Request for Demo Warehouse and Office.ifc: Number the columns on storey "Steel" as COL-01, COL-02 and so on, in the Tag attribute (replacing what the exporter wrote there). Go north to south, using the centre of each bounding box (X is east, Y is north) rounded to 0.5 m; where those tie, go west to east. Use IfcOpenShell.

First a look at what the model holds.

```python
import ifcopenshell
import ifcopenshell.util.element
import ifcopenshell.util.placement

model = ifcopenshell.open("Demo Warehouse and Office.ifc")
print(model.schema)
storey = next(s for s in model.by_type("IfcBuildingStorey") if s.Name == "Steel")
columns = [e for e in ifcopenshell.util.element.get_decomposition(storey) if e.is_a("IfcColumn")]
for e in sorted(columns, key=lambda e: e.id()):
    origin = ifcopenshell.util.placement.get_local_placement(e.ObjectPlacement)[:3, 3]
    print(e.id(), e.Tag, e.Name, origin.round(2) + 0.0, sep=" | ")
```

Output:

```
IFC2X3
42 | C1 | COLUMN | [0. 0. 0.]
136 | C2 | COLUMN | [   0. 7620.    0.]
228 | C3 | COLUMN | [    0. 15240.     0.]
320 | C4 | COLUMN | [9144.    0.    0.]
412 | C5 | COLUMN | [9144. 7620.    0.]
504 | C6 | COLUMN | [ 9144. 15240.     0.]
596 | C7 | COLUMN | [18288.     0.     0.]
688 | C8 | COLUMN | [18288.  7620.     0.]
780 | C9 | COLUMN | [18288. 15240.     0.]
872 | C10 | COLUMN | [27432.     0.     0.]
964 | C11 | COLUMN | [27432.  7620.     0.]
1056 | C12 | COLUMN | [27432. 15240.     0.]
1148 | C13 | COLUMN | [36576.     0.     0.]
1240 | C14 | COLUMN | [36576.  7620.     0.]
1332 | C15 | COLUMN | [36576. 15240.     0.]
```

```python
import ifcopenshell
import ifcopenshell.geom
import ifcopenshell.util.element
import ifcopenshell.util.shape

model = ifcopenshell.open("Demo Warehouse and Office.ifc")
settings = ifcopenshell.geom.settings()
settings.set("use-world-coords", True)


def centre(element):
    shape = ifcopenshell.geom.create_shape(settings, element)
    return ifcopenshell.util.shape.get_bbox_centroid(shape.geometry)


storey = next(s for s in model.by_type("IfcBuildingStorey") if s.Name == "Steel")
columns = [e for e in ifcopenshell.util.element.get_decomposition(storey) if e.is_a("IfcColumn")]

# Insertion points can sit at a corner or the storey origin, so sort by the geometry (in metres).
centres = {e: centre(e) for e in columns}
columns.sort(key=lambda e: (-round(centres[e][1] / 0.5), centres[e][0]))

for i, e in enumerate(columns, start=1):
    number = f"COL-{i:02d}"
    e.Tag = number
    print(e.id(), number)

model.write("Demo Warehouse and Office_rev.ifc")
```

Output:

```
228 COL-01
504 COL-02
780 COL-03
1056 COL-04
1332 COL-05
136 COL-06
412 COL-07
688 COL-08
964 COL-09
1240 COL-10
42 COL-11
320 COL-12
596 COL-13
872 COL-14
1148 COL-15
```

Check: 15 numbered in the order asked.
